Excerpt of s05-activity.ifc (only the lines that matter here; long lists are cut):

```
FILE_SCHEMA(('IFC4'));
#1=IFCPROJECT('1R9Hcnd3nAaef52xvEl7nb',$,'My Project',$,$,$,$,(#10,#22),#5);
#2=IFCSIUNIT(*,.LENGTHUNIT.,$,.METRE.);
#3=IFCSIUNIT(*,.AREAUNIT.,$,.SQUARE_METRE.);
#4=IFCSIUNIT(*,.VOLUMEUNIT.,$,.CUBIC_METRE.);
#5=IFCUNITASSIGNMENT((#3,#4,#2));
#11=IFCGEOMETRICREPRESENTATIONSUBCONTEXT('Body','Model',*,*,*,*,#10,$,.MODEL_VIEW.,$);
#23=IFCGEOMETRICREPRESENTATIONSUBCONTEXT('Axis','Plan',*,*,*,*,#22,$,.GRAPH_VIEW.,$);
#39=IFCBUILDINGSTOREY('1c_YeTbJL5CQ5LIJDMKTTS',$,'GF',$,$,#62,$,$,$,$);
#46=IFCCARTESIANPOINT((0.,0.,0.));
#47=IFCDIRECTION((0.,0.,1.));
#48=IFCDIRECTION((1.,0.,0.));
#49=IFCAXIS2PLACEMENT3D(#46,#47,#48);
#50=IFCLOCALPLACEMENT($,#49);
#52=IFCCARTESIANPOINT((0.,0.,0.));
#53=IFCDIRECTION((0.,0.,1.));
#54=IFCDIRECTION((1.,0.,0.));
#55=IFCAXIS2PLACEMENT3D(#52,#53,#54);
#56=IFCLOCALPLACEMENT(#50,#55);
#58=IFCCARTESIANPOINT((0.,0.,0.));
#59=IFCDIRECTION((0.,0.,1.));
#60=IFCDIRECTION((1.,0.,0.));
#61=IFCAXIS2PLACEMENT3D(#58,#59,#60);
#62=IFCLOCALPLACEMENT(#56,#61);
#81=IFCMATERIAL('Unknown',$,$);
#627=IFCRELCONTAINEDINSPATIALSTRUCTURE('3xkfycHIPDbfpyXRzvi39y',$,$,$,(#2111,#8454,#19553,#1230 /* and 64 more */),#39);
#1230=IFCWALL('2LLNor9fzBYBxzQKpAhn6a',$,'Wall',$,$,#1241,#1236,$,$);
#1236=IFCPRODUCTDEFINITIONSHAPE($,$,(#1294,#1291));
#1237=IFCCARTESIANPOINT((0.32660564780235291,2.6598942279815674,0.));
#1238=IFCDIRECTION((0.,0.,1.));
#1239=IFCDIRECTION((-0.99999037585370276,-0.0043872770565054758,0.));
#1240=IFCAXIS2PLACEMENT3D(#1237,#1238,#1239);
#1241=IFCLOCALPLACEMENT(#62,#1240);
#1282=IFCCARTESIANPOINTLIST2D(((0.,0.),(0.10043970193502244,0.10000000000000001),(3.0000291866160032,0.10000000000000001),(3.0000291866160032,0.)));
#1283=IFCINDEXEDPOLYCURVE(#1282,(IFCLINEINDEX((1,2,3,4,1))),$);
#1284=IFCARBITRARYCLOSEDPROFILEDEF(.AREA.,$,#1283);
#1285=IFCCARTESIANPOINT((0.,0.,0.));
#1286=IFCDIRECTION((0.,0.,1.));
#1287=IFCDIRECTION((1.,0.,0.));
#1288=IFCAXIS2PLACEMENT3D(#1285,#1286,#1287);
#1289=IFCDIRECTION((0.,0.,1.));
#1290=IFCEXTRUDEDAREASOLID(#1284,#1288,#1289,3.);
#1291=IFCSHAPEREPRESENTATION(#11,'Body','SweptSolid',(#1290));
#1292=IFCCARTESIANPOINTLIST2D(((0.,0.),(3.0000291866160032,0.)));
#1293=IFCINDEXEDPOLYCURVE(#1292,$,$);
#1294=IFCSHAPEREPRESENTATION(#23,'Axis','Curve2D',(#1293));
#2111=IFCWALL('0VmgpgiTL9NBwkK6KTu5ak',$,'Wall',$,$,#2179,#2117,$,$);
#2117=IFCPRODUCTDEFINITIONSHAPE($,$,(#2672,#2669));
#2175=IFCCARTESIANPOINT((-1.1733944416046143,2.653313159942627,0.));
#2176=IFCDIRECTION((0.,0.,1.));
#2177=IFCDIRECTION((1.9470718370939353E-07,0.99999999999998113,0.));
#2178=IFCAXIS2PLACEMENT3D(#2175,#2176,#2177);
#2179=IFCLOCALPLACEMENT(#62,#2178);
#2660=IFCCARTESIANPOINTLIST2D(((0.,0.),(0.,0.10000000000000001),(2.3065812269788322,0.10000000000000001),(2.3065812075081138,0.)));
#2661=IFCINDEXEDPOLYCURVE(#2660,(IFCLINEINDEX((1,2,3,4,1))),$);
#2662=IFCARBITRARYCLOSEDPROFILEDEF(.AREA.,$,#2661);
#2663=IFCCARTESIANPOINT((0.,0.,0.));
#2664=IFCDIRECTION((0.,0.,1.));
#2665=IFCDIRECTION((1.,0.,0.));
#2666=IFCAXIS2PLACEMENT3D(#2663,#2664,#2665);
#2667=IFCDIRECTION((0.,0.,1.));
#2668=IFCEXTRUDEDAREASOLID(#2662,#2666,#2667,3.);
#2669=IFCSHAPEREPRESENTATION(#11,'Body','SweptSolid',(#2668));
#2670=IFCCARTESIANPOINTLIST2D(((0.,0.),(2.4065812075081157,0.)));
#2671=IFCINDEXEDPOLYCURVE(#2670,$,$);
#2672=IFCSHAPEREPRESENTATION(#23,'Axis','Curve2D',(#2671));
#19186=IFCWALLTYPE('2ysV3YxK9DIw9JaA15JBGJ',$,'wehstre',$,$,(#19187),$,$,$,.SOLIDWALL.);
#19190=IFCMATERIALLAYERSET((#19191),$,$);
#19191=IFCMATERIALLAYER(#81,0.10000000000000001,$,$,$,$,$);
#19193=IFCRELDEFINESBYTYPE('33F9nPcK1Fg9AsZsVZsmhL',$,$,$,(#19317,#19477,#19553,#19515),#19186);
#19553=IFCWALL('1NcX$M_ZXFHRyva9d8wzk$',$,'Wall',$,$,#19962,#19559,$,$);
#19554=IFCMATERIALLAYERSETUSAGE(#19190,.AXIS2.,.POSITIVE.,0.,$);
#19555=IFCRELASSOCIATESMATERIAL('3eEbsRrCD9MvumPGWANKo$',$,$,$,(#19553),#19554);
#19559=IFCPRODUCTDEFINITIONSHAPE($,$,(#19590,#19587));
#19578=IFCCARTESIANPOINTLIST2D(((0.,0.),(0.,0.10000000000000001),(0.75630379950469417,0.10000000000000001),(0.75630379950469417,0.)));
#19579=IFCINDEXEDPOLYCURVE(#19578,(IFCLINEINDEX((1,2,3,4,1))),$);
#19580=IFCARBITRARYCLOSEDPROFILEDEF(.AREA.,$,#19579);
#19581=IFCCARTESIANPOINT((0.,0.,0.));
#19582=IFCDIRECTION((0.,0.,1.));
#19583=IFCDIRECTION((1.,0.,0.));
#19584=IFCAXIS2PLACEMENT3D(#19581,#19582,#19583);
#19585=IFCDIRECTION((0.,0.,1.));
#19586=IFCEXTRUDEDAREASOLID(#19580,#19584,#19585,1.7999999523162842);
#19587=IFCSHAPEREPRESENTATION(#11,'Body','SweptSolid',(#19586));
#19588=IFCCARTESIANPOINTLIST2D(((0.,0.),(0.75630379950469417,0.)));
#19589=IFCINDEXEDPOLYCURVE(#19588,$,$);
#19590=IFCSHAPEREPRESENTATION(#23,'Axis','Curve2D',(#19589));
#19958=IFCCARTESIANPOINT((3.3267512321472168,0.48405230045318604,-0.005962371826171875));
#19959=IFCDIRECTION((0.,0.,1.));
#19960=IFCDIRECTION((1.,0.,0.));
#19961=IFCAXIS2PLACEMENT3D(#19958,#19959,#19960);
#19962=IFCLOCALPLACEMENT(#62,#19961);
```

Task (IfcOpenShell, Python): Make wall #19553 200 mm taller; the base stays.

```python
import ifcopenshell
import ifcopenshell.geom
import ifcopenshell.util.representation
import ifcopenshell.util.shape
import ifcopenshell.util.unit

model = ifcopenshell.open("s05-activity.ifc")
unit_scale = ifcopenshell.util.unit.calculate_unit_scale(model)
settings = ifcopenshell.geom.settings()


def volume(element):
    """Net volume in cubic metres, openings subtracted."""
    shape = ifcopenshell.geom.create_shape(settings, element)
    return ifcopenshell.util.shape.get_volume(shape.geometry)


wall = model.by_guid("1NcX$M_ZXFHRyva9d8wzk$")
before = volume(wall)

body = ifcopenshell.util.representation.get_representation(wall, "Model", "Body")
solid = body.Items[0]
old_height = solid.Depth
solid.Depth += 0.2 / unit_scale
after = volume(wall)

print(f"height {old_height:g} -> {solid.Depth:g}, volume {before:.3f} -> {after:.3f} m3")

model.write("s05-activity_updated.ifc")
```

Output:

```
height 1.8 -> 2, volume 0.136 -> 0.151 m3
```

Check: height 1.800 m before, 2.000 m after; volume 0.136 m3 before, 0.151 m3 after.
